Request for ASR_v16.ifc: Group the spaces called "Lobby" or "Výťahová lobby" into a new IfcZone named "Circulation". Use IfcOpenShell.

First a look at what the model holds.

```python
import ifcopenshell

model = ifcopenshell.open("ASR_v16.ifc")
print(model.schema)
seen = {}
for space in model.by_type("IfcSpace"):
    seen[space.LongName] = seen.get(space.LongName, 0) + 1
for name, count in sorted(seen.items(), key=str):
    print(count, "x", name)
print("zones:", [z.Name for z in model.by_type("IfcZone")][:20])
```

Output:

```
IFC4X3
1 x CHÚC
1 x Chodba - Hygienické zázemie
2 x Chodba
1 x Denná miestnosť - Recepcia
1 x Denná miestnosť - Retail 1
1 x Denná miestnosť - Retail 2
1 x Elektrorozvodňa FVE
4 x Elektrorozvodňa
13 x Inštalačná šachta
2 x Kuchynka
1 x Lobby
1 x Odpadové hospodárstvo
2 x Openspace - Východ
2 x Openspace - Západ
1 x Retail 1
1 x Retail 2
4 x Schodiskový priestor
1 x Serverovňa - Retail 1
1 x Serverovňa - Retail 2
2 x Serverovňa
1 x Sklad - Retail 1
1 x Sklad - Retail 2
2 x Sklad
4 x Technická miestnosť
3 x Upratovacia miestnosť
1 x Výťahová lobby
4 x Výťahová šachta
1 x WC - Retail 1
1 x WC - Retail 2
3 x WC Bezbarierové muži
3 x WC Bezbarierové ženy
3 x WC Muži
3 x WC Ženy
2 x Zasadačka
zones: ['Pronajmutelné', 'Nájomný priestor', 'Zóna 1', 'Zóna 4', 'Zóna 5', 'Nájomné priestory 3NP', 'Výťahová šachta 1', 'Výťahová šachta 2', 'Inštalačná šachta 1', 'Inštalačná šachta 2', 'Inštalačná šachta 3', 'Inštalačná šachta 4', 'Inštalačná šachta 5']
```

```python
import ifcopenshell
import ifcopenshell.api.group
import ifcopenshell.api.root

model = ifcopenshell.open("ASR_v16.ifc")

names = {"Lobby", "Výťahová lobby"}
spaces = [s for s in model.by_type("IfcSpace") if s.LongName in names]

zone = ifcopenshell.api.root.create_entity(model, ifc_class="IfcZone", name="Circulation")
ifcopenshell.api.group.assign_group(model, products=spaces, group=zone)
print(len(spaces), "spaces in", zone.Name)

model.write("ASR_v16-out.ifc")
```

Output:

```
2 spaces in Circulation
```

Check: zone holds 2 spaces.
